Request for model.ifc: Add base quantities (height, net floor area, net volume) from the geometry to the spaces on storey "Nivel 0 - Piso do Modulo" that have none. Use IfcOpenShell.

First a look at what the model holds.

```python
import ifcopenshell
import ifcopenshell.util.element
import ifcopenshell.util.unit

model = ifcopenshell.open("model.ifc")
print(model.schema)
for unit_type in ("LENGTHUNIT", "AREAUNIT", "VOLUMEUNIT"):
    print(unit_type, ifcopenshell.util.unit.calculate_unit_scale(model, unit_type))
storey = next(s for s in model.by_type("IfcBuildingStorey") if s.Name == "Nivel 0 - Piso do Modulo")
spaces = [e for e in ifcopenshell.util.element.get_decomposition(storey) if e.is_a("IfcSpace")]
for e in sorted(spaces, key=lambda e: e.id()):
    print(e.id(), e.is_a(), e.Name, list(ifcopenshell.util.element.get_psets(e, qtos_only=True)), sep=" | ")
```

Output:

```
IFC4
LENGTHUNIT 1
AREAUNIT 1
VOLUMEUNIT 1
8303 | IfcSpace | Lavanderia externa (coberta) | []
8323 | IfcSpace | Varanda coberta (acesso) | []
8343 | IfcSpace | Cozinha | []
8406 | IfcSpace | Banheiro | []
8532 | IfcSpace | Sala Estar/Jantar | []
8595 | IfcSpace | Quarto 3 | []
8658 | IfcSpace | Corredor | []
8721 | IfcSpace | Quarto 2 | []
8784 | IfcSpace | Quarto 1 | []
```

```python
import ifcopenshell
import ifcopenshell.api.pset
import ifcopenshell.geom
import ifcopenshell.util.element
import ifcopenshell.util.shape
import ifcopenshell.util.unit

model = ifcopenshell.open("model.ifc")
unit_scale = ifcopenshell.util.unit.calculate_unit_scale(model)
area_scale = ifcopenshell.util.unit.calculate_unit_scale(model, "AREAUNIT")
volume_scale = ifcopenshell.util.unit.calculate_unit_scale(model, "VOLUMEUNIT")
settings = ifcopenshell.geom.settings()

storey = next(s for s in model.by_type("IfcBuildingStorey") if s.Name == "Nivel 0 - Piso do Modulo")
spaces = [e for e in ifcopenshell.util.element.get_decomposition(storey) if e.is_a("IfcSpace")]

for e in sorted(spaces, key=lambda e: e.id()):
    if ifcopenshell.util.element.get_psets(e, qtos_only=True, should_inherit=False):
        continue
    # Geometry comes back in metres, in the element's own axes.
    shape = ifcopenshell.geom.create_shape(settings, e)
    values = {
        "Height": ifcopenshell.util.shape.get_z(shape.geometry) / unit_scale,
        "NetFloorArea": ifcopenshell.util.shape.get_footprint_area(shape.geometry) / area_scale,
        "NetVolume": ifcopenshell.util.shape.get_volume(shape.geometry) / volume_scale,
    }
    qto = ifcopenshell.api.pset.add_qto(model, product=e, name="Qto_SpaceBaseQuantities")
    ifcopenshell.api.pset.edit_qto(model, qto=qto, properties=values)
    print(e.id(), {k: round(v, 3) for k, v in values.items()})

model.write("model_edited.ifc")
```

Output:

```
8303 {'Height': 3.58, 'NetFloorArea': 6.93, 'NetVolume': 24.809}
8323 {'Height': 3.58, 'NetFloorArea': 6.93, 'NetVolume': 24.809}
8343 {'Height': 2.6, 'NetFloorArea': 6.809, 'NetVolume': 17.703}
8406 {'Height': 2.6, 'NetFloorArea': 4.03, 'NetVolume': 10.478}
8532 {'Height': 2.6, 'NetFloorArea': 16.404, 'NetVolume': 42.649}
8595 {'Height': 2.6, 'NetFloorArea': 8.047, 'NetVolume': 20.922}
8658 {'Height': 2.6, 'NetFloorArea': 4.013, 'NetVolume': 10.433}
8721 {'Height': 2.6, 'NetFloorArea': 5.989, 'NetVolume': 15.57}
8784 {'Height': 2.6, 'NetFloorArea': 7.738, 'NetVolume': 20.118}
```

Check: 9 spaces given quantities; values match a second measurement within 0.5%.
